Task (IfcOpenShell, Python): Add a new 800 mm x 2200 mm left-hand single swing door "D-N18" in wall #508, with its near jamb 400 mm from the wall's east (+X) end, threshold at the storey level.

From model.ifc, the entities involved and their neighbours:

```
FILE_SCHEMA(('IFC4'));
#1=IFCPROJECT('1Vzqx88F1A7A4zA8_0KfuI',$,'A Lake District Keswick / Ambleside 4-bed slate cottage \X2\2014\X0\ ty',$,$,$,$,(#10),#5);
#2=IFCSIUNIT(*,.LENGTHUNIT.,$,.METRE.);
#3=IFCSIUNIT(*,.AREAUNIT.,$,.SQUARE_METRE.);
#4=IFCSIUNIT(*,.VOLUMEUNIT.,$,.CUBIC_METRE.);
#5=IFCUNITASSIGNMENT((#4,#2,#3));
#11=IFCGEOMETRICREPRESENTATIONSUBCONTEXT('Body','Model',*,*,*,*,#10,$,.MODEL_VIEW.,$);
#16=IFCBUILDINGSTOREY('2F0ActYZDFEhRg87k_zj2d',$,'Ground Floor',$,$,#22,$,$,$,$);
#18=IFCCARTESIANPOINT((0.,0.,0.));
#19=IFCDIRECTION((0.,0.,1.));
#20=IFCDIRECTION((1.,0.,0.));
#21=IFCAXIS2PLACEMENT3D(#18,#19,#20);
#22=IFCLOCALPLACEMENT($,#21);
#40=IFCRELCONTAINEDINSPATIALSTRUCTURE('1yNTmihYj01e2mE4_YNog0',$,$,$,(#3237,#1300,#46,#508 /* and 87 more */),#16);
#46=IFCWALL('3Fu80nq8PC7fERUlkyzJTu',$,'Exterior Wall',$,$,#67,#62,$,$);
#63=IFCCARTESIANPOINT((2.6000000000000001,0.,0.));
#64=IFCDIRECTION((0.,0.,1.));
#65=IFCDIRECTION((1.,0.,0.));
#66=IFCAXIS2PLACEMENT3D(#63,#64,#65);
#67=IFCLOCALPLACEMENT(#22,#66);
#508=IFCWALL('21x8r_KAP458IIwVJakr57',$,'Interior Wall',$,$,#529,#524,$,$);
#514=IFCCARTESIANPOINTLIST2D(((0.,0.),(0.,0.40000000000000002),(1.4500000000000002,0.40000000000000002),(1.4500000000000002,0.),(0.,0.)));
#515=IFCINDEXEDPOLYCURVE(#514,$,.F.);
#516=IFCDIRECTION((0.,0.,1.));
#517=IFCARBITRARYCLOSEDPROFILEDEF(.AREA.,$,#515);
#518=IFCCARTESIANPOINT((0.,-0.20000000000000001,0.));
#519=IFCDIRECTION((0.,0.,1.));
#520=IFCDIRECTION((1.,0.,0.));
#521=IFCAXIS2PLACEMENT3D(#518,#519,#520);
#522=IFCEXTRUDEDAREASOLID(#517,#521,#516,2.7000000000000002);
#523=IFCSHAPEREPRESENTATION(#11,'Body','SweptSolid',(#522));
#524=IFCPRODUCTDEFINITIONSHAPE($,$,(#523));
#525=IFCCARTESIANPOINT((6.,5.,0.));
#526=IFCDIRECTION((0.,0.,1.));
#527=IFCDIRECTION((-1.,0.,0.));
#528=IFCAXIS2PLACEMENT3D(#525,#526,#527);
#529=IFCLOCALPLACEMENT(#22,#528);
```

```python
import numpy as np
import ifcopenshell
import ifcopenshell.api.feature
import ifcopenshell.api.geometry
import ifcopenshell.api.root
import ifcopenshell.api.spatial
import ifcopenshell.geom
import ifcopenshell.util.element
import ifcopenshell.util.placement
import ifcopenshell.util.representation
import ifcopenshell.util.shape
import ifcopenshell.util.unit

model = ifcopenshell.open("model.ifc")
unit_scale = ifcopenshell.util.unit.calculate_unit_scale(model)
settings = ifcopenshell.geom.settings()


def volume(element):
    """Net volume in cubic metres, openings subtracted."""
    shape = ifcopenshell.geom.create_shape(settings, element)
    return ifcopenshell.util.shape.get_volume(shape.geometry)


wall = model.by_guid("21x8r_KAP458IIwVJakr57")
storey = ifcopenshell.util.element.get_container(wall, ifc_class="IfcBuildingStorey")
context = ifcopenshell.util.representation.get_context(model, "Model", "Body", "MODEL_VIEW")
before = volume(wall)

width, height, from_end, sill = 0.8, 2.2, 0.4, 0.0  # metres

# The wall runs along its own X axis, and the end named is its -X end.
wall_shape = ifcopenshell.geom.create_shape(settings, wall)
x, y, z = ifcopenshell.util.shape.get_vertices(wall_shape.geometry).T
start = x.min() + from_end
face, thickness = float(y.min()), float(y.max() - y.min())
wall_matrix = ifcopenshell.util.placement.get_local_placement(wall.ObjectPlacement)
level = ifcopenshell.util.placement.get_local_placement(storey.ObjectPlacement)[2, 3]


def in_wall(x, y):
    """Placement at x, y metres in the wall's axes, at sill height."""
    matrix = wall_matrix.copy()
    matrix[:, 3] = wall_matrix @ np.array([x / unit_scale, y / unit_scale, 0.0, 1.0])
    matrix[2, 3] = level + sill / unit_scale
    return matrix


# Opening: a box that overshoots both wall faces by 50 mm.
opening = ifcopenshell.api.root.create_entity(model, ifc_class="IfcOpeningElement", predefined_type="OPENING")
box = ifcopenshell.api.geometry.add_wall_representation(
    model, context=context, length=width, height=height, thickness=thickness + 0.1
)
ifcopenshell.api.geometry.assign_representation(model, product=opening, representation=box)
ifcopenshell.api.geometry.edit_object_placement(model, product=opening, matrix=in_wall(start, face - 0.05), is_si=False)
ifcopenshell.api.feature.add_feature(model, feature=opening, element=wall)

door = ifcopenshell.api.root.create_entity(model, ifc_class="IfcDoor", name="D-N18", predefined_type="DOOR")
door.OverallWidth, door.OverallHeight = width / unit_scale, height / unit_scale
door.OperationType = "SINGLE_SWING_LEFT"
body = ifcopenshell.api.geometry.add_door_representation(
    model,
    context=context,
    overall_width=door.OverallWidth,
    overall_height=door.OverallHeight,
    operation_type="SINGLE_SWING_LEFT",
    lining_properties={"LiningDepth": thickness / unit_scale, "ThresholdDepth": thickness / unit_scale},
)
ifcopenshell.api.geometry.assign_representation(model, product=door, representation=body)
ifcopenshell.api.spatial.assign_container(model, products=[door], relating_structure=storey)
ifcopenshell.api.feature.add_filling(model, opening=opening, element=door)

# The lining spans the wall, so the door starts at the wall face.
ifcopenshell.api.geometry.edit_object_placement(model, product=door, matrix=in_wall(start, face), is_si=False)

after = volume(wall)

print(f"wall volume {before:.3f} -> {after:.3f} m3")

model.write("model_v2.ifc")
```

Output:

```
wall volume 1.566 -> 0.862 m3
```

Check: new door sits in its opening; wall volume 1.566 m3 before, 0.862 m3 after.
